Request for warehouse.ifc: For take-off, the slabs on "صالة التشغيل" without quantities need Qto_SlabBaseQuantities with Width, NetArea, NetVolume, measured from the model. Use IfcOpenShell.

First a look at what the model holds.

```python
import ifcopenshell
import ifcopenshell.util.element
import ifcopenshell.util.unit

model = ifcopenshell.open("warehouse.ifc")
print(model.schema)
for unit_type in ("LENGTHUNIT", "AREAUNIT", "VOLUMEUNIT"):
    print(unit_type, ifcopenshell.util.unit.calculate_unit_scale(model, unit_type))
storey = next(s for s in model.by_type("IfcBuildingStorey") if s.Name == "صالة التشغيل")
slabs = [e for e in ifcopenshell.util.element.get_decomposition(storey) if e.is_a("IfcSlab")]
for e in sorted(slabs, key=lambda e: e.id()):
    print(e.id(), e.is_a(), e.Name, list(ifcopenshell.util.element.get_psets(e, qtos_only=True)), sep=" | ")
```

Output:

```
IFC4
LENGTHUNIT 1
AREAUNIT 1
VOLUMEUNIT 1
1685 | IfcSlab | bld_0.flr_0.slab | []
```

```python
import ifcopenshell
import ifcopenshell.api.pset
import ifcopenshell.geom
import ifcopenshell.util.element
import ifcopenshell.util.shape
import ifcopenshell.util.unit

model = ifcopenshell.open("warehouse.ifc")
unit_scale = ifcopenshell.util.unit.calculate_unit_scale(model)
area_scale = ifcopenshell.util.unit.calculate_unit_scale(model, "AREAUNIT")
volume_scale = ifcopenshell.util.unit.calculate_unit_scale(model, "VOLUMEUNIT")
settings = ifcopenshell.geom.settings()

storey = next(s for s in model.by_type("IfcBuildingStorey") if s.Name == "صالة التشغيل")
slabs = [e for e in ifcopenshell.util.element.get_decomposition(storey) if e.is_a("IfcSlab")]

for e in sorted(slabs, key=lambda e: e.id()):
    if ifcopenshell.util.element.get_psets(e, qtos_only=True, should_inherit=False):
        continue
    # Geometry comes back in metres, in the element's own axes.
    shape = ifcopenshell.geom.create_shape(settings, e)
    values = {
        "Width": ifcopenshell.util.shape.get_z(shape.geometry) / unit_scale,
        "NetArea": ifcopenshell.util.shape.get_footprint_area(shape.geometry) / area_scale,
        "NetVolume": ifcopenshell.util.shape.get_volume(shape.geometry) / volume_scale,
    }
    qto = ifcopenshell.api.pset.add_qto(model, product=e, name="Qto_SlabBaseQuantities")
    ifcopenshell.api.pset.edit_qto(model, qto=qto, properties=values)
    print(e.id(), {k: round(v, 3) for k, v in values.items()})

model.write("warehouse-out.ifc")
```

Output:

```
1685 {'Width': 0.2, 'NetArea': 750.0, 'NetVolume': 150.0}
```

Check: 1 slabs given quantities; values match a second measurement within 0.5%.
